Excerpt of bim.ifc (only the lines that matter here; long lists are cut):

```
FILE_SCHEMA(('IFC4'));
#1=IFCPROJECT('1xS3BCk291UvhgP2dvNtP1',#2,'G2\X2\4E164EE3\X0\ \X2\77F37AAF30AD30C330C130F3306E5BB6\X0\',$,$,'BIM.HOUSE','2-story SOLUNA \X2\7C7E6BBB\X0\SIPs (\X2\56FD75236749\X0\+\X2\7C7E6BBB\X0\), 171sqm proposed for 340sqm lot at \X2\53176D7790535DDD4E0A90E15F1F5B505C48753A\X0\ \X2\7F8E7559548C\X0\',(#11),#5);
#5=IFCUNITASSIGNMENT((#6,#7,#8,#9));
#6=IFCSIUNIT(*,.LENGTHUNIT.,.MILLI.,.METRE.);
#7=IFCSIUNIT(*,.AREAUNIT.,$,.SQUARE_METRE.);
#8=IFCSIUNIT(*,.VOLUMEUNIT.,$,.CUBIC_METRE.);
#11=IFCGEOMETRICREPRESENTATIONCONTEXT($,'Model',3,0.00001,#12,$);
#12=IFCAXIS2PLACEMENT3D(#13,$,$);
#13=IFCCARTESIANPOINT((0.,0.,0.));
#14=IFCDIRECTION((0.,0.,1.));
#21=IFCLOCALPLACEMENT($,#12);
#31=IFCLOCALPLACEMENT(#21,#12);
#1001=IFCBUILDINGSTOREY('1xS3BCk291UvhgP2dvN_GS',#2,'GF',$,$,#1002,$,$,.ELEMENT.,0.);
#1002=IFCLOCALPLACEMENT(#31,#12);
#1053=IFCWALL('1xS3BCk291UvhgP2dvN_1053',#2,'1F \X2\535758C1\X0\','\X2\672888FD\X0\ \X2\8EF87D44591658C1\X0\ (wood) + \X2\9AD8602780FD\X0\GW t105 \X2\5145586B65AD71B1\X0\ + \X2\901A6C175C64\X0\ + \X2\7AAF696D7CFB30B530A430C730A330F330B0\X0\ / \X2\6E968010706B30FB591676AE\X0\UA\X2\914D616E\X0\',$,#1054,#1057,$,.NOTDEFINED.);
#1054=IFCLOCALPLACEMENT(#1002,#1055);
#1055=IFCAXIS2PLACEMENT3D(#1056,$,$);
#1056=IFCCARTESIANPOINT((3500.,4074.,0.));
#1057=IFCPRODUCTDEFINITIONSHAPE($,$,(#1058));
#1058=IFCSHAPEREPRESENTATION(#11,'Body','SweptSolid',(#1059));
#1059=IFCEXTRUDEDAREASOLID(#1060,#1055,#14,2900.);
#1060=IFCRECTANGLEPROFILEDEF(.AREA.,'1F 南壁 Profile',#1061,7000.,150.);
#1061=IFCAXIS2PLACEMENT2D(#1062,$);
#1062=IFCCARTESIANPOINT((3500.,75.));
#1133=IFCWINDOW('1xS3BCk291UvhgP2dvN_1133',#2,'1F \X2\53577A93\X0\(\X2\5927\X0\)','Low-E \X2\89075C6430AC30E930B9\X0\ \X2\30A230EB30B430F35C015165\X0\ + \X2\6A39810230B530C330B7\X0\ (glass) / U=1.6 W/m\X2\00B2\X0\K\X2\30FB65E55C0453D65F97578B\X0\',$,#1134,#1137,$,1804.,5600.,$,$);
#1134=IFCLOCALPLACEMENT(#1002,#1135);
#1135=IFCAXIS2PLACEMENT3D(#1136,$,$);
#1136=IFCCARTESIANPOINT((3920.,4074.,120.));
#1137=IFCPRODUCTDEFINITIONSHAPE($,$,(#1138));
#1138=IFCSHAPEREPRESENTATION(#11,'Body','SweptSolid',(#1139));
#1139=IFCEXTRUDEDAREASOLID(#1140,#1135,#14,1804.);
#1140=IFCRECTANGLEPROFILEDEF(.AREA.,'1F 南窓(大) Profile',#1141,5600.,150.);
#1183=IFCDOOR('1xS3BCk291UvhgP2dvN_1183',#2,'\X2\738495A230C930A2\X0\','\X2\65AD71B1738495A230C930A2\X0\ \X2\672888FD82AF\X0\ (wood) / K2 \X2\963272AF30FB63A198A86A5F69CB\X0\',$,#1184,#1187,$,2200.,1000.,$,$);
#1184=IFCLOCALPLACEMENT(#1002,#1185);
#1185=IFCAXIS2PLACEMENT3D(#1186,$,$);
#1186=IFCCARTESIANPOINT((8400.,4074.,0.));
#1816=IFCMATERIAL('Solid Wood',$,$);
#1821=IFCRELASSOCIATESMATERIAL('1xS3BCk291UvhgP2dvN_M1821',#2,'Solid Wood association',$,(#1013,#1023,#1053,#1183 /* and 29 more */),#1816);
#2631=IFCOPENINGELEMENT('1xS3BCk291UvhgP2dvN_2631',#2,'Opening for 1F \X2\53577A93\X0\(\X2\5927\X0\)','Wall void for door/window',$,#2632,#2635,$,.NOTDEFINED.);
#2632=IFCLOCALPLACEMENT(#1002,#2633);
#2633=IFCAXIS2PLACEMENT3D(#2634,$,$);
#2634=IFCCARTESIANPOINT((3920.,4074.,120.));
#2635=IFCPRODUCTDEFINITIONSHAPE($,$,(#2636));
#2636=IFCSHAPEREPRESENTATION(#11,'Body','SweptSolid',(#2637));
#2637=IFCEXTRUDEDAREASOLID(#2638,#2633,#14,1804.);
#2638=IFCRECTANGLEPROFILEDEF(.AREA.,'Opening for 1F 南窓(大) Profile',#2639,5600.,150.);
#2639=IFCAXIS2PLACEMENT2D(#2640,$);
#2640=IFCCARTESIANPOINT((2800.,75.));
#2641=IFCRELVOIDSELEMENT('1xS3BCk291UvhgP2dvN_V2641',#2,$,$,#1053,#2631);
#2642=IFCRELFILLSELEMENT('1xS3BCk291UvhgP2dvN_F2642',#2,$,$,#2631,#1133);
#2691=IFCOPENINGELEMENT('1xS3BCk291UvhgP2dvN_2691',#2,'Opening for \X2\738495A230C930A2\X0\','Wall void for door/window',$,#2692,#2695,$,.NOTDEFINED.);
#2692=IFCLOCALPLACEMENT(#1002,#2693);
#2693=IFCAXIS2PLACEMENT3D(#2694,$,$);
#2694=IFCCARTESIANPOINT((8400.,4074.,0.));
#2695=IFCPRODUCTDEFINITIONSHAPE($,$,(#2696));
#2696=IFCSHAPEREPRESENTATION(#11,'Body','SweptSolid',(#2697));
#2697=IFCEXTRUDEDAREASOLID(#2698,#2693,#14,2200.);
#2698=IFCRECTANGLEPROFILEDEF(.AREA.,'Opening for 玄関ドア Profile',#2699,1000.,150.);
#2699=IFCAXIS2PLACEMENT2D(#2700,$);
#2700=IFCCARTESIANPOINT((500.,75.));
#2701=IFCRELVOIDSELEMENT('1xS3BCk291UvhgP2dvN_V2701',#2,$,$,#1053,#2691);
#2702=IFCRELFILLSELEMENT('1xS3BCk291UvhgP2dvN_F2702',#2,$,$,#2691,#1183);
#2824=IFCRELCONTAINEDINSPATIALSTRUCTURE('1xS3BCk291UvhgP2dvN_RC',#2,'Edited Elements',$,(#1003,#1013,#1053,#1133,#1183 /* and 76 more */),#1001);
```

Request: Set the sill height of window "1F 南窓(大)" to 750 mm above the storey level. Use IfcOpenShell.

```python
import numpy as np
import ifcopenshell
import ifcopenshell.api.geometry
import ifcopenshell.geom
import ifcopenshell.util.element
import ifcopenshell.util.placement
import ifcopenshell.util.shape
import ifcopenshell.util.unit

model = ifcopenshell.open("bim.ifc")
unit_scale = ifcopenshell.util.unit.calculate_unit_scale(model)

window = model.by_id(1133)
opening = window.FillsVoids[0].RelatingOpeningElement
storey = ifcopenshell.util.element.get_container(window, ifc_class="IfcBuildingStorey")
level = ifcopenshell.util.placement.get_local_placement(storey.ObjectPlacement)[2, 3]

# The opening's origin need not be at the sill, so measure its lowest point.
shape = ifcopenshell.geom.create_shape(ifcopenshell.geom.settings(), opening)
bottom = ifcopenshell.util.shape.get_shape_bottom_elevation(shape, shape.geometry) / unit_scale
dz = level + 0.75 / unit_scale - bottom

shift = np.array([0.0, 0.0, dz])
# The window is not placed relative to its opening, so move both.
for product in (opening, window):
    matrix = ifcopenshell.util.placement.get_local_placement(product.ObjectPlacement)
    matrix[:3, 3] += shift
    ifcopenshell.api.geometry.edit_object_placement(model, product=product, matrix=matrix, is_si=False)

print(f"moved by {dz * unit_scale:+.3f} m")

model.write("bim_updated.ifc")
```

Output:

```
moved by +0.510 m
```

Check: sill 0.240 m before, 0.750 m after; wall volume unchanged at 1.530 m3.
